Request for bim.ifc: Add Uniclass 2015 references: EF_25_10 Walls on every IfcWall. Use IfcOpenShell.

First a look at what the model holds.

```python
import ifcopenshell

model = ifcopenshell.open("bim.ifc")
print(model.schema)
print("classifications:", [c.Name for c in model.by_type("IfcClassification")])
for ifc_class in ("IfcDoor", "IfcRoof", "IfcStair", "IfcWall", "IfcWindow"):
    print(ifc_class, len(model.by_type(ifc_class)))
```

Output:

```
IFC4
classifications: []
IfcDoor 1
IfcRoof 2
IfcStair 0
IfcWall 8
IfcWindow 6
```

```python
import ifcopenshell
import ifcopenshell.api.classification

model = ifcopenshell.open("bim.ifc")

system = ifcopenshell.api.classification.add_classification(model, classification="Uniclass 2015")

codes = {
    "IfcWall": ("EF_25_10", "Walls"),
}
for ifc_class, (code, name) in codes.items():
    products = model.by_type(ifc_class)
    ifcopenshell.api.classification.add_reference(
        model, products=products, classification=system, identification=code, name=name
    )
    print(code, len(products))

model.write("bim-out.ifc")
```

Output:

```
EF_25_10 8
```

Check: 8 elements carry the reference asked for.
